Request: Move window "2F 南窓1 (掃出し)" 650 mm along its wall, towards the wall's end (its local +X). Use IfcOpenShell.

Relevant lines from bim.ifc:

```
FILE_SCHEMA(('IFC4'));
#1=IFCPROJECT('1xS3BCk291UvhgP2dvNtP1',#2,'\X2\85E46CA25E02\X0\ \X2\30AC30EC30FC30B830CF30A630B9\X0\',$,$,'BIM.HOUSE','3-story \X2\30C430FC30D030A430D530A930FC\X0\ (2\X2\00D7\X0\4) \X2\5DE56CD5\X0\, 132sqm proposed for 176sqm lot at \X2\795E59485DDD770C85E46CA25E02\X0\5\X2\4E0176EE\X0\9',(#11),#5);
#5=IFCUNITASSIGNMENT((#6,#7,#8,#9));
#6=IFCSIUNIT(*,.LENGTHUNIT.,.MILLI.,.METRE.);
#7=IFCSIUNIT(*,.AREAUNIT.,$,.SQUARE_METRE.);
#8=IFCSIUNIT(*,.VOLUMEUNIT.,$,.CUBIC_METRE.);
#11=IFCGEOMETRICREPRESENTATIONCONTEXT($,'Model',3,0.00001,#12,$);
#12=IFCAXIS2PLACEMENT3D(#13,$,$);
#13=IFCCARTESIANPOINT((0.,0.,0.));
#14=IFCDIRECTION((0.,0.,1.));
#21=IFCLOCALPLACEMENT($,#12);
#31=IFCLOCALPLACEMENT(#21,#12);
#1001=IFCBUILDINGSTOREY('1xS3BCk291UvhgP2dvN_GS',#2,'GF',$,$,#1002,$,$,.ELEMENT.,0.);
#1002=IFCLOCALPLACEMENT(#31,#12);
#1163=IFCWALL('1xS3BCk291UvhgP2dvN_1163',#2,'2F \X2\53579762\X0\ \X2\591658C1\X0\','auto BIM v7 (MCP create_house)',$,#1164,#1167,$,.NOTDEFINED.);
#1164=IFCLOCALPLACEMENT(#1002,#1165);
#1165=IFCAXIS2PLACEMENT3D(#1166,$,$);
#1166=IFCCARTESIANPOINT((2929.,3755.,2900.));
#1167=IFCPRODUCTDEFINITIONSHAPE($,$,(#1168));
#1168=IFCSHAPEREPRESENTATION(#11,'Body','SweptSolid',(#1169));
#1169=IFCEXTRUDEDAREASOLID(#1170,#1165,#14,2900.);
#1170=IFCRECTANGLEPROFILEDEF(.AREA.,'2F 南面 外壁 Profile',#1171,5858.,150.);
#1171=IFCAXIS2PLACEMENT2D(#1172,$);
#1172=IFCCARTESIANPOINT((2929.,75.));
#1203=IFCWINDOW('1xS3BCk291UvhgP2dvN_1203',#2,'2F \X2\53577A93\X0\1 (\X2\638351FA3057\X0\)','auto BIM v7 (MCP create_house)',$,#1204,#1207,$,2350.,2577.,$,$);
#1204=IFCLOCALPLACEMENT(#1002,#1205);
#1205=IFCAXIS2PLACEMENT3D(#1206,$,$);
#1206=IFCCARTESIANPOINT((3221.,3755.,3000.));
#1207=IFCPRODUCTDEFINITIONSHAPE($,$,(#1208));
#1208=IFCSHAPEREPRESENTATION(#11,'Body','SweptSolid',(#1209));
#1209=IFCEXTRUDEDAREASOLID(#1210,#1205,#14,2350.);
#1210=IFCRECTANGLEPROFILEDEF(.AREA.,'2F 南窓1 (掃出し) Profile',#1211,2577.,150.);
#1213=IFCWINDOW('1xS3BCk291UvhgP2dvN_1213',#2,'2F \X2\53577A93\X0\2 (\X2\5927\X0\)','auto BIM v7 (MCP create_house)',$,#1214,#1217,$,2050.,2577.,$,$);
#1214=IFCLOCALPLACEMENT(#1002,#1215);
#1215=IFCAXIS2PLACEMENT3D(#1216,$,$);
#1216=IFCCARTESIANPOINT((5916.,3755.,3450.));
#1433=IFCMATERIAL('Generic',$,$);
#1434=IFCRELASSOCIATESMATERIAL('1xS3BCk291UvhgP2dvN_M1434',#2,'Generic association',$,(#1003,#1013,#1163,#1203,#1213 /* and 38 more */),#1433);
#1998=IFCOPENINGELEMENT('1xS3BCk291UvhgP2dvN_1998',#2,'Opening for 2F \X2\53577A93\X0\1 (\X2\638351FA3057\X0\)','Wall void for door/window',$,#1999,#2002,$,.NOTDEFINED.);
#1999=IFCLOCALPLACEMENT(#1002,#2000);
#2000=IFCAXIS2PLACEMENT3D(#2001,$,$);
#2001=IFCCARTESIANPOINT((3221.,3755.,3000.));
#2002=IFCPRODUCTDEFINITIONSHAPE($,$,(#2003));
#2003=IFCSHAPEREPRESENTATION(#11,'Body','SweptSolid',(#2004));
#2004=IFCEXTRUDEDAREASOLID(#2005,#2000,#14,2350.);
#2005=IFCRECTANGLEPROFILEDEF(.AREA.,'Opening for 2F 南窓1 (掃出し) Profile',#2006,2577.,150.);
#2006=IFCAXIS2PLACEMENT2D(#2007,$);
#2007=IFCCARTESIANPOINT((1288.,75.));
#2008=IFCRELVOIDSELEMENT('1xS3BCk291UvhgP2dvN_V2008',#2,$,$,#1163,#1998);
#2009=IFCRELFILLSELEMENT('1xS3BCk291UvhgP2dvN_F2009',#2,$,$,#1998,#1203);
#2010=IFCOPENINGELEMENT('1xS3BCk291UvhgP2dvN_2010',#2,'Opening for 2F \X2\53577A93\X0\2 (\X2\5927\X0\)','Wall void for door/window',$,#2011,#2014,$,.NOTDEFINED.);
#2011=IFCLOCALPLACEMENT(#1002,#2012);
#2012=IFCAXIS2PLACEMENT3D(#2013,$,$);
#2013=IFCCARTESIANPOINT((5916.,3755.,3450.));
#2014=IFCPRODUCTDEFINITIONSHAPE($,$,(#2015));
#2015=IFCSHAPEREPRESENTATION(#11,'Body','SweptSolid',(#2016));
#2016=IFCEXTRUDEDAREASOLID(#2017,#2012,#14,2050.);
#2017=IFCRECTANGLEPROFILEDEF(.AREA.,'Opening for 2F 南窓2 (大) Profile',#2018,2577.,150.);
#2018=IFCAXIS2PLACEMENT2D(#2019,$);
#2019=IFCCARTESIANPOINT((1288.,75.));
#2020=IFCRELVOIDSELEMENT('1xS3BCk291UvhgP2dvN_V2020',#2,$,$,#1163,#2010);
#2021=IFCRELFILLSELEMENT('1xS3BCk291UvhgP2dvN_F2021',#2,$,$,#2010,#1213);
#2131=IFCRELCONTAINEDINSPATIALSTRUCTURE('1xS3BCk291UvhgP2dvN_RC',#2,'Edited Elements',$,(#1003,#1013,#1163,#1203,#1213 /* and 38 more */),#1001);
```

```python
import ifcopenshell
import ifcopenshell.api.geometry
import ifcopenshell.util.placement
import ifcopenshell.util.unit

model = ifcopenshell.open("bim.ifc")
unit_scale = ifcopenshell.util.unit.calculate_unit_scale(model)

window = model.by_guid("1xS3BCk291UvhgP2dvN_1203")
opening = window.FillsVoids[0].RelatingOpeningElement
wall = opening.VoidsElements[0].RelatingBuildingElement

wall_matrix = ifcopenshell.util.placement.get_local_placement(wall.ObjectPlacement)
shift = wall_matrix[:3, 0] * 0.65 / unit_scale
before = ifcopenshell.util.placement.get_local_placement(window.ObjectPlacement)[:3, 3].copy()

# The window is not placed relative to its opening, so move both.
for product in (opening, window):
    matrix = ifcopenshell.util.placement.get_local_placement(product.ObjectPlacement)
    matrix[:3, 3] += shift
    ifcopenshell.api.geometry.edit_object_placement(model, product=product, matrix=matrix, is_si=False)

after = ifcopenshell.util.placement.get_local_placement(window.ObjectPlacement)[:3, 3]
print("window moved by", (after - before).round(3) + 0.0)

model.write("bim_edited.ifc")
```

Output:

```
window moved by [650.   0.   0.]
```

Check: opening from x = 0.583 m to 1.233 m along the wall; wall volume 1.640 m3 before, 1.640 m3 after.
